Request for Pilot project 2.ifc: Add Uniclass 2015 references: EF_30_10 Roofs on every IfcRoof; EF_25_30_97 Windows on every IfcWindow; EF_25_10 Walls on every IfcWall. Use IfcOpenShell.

First a look at what the model holds.

```python
import ifcopenshell

model = ifcopenshell.open("Pilot project 2.ifc")
print(model.schema)
print("classifications:", [c.Name for c in model.by_type("IfcClassification")])
for ifc_class in ("IfcDoor", "IfcRoof", "IfcStair", "IfcWall", "IfcWindow"):
    print(ifc_class, len(model.by_type(ifc_class)))
```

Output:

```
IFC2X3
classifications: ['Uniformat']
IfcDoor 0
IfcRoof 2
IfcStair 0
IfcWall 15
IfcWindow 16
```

```python
import ifcopenshell
import ifcopenshell.api.classification

model = ifcopenshell.open("Pilot project 2.ifc")

# IFC2X3 requires Source and Edition and has no link from the project to the system.
system = model.create_entity("IfcClassification", Source="NBS", Edition="2015", Name="Uniclass 2015")

codes = {
    "IfcRoof": ("EF_30_10", "Roofs"),
    "IfcWindow": ("EF_25_30_97", "Windows"),
    "IfcWall": ("EF_25_10", "Walls"),
}
for ifc_class, (code, name) in codes.items():
    products = model.by_type(ifc_class)
    ifcopenshell.api.classification.add_reference(
        model, products=products, classification=system, identification=code, name=name
    )
    print(code, len(products))

model.write("Pilot project 2_rev.ifc")
```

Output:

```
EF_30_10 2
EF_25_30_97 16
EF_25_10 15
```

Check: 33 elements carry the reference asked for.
